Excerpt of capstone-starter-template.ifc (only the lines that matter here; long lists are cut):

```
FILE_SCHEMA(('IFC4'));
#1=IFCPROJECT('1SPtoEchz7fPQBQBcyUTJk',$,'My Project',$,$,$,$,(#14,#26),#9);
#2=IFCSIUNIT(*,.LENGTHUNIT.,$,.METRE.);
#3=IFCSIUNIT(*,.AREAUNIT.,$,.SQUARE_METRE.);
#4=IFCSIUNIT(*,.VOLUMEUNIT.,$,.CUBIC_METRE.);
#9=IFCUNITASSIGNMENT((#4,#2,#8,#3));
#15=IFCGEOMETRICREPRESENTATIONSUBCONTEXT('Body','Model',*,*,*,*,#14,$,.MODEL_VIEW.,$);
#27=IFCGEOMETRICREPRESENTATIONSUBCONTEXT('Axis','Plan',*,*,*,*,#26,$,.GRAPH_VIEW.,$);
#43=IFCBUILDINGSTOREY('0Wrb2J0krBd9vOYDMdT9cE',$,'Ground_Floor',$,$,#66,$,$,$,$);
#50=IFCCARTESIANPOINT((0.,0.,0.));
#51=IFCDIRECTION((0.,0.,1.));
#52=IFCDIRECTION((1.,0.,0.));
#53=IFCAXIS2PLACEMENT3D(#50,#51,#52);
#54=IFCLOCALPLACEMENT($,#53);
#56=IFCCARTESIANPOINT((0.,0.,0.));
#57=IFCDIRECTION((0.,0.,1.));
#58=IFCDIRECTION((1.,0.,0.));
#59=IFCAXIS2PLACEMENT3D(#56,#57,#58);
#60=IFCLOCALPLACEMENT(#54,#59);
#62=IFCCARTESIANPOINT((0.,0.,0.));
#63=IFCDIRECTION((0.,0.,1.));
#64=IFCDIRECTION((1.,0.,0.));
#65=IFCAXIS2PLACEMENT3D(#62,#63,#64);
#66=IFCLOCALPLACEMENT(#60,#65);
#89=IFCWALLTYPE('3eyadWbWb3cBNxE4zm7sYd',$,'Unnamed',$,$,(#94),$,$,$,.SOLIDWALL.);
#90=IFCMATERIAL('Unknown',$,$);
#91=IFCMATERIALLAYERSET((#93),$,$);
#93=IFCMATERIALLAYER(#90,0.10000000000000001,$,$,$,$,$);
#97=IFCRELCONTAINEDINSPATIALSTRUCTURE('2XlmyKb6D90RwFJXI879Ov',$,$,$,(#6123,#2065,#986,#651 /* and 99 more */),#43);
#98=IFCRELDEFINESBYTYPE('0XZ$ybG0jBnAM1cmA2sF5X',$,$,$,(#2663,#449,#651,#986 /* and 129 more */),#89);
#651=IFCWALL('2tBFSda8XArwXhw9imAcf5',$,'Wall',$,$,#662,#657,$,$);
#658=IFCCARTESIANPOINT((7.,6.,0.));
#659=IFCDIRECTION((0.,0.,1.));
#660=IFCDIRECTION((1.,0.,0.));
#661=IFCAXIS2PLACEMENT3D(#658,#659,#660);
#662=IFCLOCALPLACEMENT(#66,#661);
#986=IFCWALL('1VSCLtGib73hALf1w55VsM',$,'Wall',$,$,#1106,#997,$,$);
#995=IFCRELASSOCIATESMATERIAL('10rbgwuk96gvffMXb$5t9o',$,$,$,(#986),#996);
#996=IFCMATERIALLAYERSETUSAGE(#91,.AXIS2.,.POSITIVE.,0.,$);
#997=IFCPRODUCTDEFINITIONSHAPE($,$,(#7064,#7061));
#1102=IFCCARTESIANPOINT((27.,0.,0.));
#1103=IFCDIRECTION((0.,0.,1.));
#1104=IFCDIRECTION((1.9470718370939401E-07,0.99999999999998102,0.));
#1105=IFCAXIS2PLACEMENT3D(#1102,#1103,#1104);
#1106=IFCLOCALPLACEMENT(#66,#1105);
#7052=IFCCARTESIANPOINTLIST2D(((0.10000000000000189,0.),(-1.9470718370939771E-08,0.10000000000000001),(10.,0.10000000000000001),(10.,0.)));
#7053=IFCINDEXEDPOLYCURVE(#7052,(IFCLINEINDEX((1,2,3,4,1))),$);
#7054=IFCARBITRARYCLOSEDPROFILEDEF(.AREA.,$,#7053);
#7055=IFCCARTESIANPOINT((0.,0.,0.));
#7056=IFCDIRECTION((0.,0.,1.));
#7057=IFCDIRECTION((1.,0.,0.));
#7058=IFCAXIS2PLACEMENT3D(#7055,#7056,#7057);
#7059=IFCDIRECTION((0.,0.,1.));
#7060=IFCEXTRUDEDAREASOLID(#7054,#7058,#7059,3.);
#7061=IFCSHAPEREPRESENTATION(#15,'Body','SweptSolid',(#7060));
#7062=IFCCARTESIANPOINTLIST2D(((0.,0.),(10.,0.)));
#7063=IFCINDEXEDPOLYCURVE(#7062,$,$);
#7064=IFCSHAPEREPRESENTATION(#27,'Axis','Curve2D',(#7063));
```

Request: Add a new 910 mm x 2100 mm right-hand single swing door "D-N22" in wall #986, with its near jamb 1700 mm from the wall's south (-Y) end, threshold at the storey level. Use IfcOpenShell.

```python
import numpy as np
import ifcopenshell
import ifcopenshell.api.feature
import ifcopenshell.api.geometry
import ifcopenshell.api.root
import ifcopenshell.api.spatial
import ifcopenshell.geom
import ifcopenshell.util.element
import ifcopenshell.util.placement
import ifcopenshell.util.representation
import ifcopenshell.util.shape
import ifcopenshell.util.unit

model = ifcopenshell.open("capstone-starter-template.ifc")
unit_scale = ifcopenshell.util.unit.calculate_unit_scale(model)
settings = ifcopenshell.geom.settings()


def volume(element):
    """Net volume in cubic metres, openings subtracted."""
    shape = ifcopenshell.geom.create_shape(settings, element)
    return ifcopenshell.util.shape.get_volume(shape.geometry)


wall = model.by_guid("1VSCLtGib73hALf1w55VsM")
storey = ifcopenshell.util.element.get_container(wall, ifc_class="IfcBuildingStorey")
context = ifcopenshell.util.representation.get_context(model, "Model", "Body", "MODEL_VIEW")
before = volume(wall)

width, height, from_end, sill = 0.91, 2.1, 1.7, 0.0  # metres

# The wall runs along its own X axis, and the end named is its -X end.
wall_shape = ifcopenshell.geom.create_shape(settings, wall)
x, y, z = ifcopenshell.util.shape.get_vertices(wall_shape.geometry).T
start = x.min() + from_end
face, thickness = float(y.min()), float(y.max() - y.min())
wall_matrix = ifcopenshell.util.placement.get_local_placement(wall.ObjectPlacement)
level = ifcopenshell.util.placement.get_local_placement(storey.ObjectPlacement)[2, 3]


def in_wall(x, y):
    """Placement at x, y metres in the wall's axes, at sill height."""
    matrix = wall_matrix.copy()
    matrix[:, 3] = wall_matrix @ np.array([x / unit_scale, y / unit_scale, 0.0, 1.0])
    matrix[2, 3] = level + sill / unit_scale
    return matrix


# Opening: a box that overshoots both wall faces by 50 mm.
opening = ifcopenshell.api.root.create_entity(model, ifc_class="IfcOpeningElement", predefined_type="OPENING")
box = ifcopenshell.api.geometry.add_wall_representation(
    model, context=context, length=width, height=height, thickness=thickness + 0.1
)
ifcopenshell.api.geometry.assign_representation(model, product=opening, representation=box)
ifcopenshell.api.geometry.edit_object_placement(model, product=opening, matrix=in_wall(start, face - 0.05), is_si=False)
ifcopenshell.api.feature.add_feature(model, feature=opening, element=wall)

door = ifcopenshell.api.root.create_entity(model, ifc_class="IfcDoor", name="D-N22", predefined_type="DOOR")
door.OverallWidth, door.OverallHeight = width / unit_scale, height / unit_scale
door.OperationType = "SINGLE_SWING_RIGHT"
body = ifcopenshell.api.geometry.add_door_representation(
    model,
    context=context,
    overall_width=door.OverallWidth,
    overall_height=door.OverallHeight,
    operation_type="SINGLE_SWING_RIGHT",
    lining_properties={"LiningDepth": thickness / unit_scale, "ThresholdDepth": thickness / unit_scale},
)
ifcopenshell.api.geometry.assign_representation(model, product=door, representation=body)
ifcopenshell.api.spatial.assign_container(model, products=[door], relating_structure=storey)
ifcopenshell.api.feature.add_filling(model, opening=opening, element=door)

# The lining spans the wall, so the door starts at the wall face.
ifcopenshell.api.geometry.edit_object_placement(model, product=door, matrix=in_wall(start, face), is_si=False)

after = volume(wall)

print(f"wall volume {before:.3f} -> {after:.3f} m3")

model.write("capstone-starter-template_rev.ifc")
```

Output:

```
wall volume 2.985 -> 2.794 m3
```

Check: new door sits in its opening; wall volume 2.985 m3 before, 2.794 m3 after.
